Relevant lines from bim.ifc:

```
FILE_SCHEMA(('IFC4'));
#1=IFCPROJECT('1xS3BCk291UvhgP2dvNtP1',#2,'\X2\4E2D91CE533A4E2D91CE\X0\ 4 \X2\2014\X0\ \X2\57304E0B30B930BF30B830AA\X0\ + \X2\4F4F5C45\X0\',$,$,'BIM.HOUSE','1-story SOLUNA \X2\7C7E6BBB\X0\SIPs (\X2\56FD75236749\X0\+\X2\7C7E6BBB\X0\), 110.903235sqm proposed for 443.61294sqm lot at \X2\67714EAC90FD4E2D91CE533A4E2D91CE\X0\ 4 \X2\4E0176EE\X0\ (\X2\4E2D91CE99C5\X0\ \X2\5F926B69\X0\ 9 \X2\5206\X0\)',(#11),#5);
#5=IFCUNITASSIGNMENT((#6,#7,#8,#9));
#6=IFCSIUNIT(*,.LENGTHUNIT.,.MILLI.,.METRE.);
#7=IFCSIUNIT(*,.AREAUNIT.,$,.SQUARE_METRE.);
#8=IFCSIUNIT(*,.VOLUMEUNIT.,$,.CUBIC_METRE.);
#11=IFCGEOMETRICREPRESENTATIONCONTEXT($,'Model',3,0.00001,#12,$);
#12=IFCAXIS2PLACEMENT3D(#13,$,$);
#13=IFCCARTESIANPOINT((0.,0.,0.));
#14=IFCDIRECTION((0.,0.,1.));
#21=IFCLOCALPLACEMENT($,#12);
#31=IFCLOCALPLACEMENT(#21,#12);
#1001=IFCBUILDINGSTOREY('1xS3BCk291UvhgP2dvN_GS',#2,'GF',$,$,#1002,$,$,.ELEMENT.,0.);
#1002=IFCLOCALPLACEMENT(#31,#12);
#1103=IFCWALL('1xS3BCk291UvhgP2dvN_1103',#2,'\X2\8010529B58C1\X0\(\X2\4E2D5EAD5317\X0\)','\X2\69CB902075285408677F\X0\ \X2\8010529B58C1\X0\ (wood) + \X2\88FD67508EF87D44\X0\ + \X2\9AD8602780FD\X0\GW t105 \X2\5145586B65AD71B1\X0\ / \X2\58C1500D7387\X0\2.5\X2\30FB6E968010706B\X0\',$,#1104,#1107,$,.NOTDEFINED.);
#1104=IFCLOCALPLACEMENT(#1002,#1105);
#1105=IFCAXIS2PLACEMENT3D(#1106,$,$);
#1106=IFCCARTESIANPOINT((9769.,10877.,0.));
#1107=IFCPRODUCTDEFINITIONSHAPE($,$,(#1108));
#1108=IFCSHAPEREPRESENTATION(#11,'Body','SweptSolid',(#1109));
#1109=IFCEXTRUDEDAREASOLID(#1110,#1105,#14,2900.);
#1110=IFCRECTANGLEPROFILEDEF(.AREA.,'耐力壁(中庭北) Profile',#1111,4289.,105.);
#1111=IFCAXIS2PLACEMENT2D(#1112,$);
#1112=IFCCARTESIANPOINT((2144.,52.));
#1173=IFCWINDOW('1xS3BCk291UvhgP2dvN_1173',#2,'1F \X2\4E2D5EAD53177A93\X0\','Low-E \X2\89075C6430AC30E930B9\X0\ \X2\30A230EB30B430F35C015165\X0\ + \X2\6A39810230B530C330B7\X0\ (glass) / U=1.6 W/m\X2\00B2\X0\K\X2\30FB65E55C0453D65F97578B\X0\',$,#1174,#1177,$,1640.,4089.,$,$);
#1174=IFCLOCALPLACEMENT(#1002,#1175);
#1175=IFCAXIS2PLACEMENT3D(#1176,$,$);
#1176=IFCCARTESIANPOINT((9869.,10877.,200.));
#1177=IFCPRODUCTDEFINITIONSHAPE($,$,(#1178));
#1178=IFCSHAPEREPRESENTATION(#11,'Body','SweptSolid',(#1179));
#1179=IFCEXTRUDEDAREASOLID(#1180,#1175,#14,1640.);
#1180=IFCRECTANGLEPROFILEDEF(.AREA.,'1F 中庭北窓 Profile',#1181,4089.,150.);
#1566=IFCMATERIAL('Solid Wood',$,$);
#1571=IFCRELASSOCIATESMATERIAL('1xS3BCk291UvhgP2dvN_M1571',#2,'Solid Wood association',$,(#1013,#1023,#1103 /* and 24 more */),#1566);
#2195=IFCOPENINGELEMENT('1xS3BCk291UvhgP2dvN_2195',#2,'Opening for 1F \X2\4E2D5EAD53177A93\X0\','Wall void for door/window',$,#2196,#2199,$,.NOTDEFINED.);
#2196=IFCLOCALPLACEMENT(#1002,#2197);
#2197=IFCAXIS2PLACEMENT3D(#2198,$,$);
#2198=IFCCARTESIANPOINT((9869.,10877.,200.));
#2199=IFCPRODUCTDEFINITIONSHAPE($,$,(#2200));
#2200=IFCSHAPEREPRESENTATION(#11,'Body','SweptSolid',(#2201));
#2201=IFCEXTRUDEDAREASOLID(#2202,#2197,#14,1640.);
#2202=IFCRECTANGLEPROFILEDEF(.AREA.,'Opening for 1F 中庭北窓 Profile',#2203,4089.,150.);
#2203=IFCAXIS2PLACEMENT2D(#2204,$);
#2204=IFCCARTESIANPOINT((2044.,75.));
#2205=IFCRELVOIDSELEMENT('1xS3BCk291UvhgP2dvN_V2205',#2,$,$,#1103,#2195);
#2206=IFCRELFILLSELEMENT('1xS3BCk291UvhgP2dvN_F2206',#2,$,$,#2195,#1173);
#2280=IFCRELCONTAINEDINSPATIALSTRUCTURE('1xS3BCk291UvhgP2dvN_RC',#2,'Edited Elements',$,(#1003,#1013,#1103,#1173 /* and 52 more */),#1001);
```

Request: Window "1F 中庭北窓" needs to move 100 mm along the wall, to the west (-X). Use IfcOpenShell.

```python
import ifcopenshell
import ifcopenshell.api.geometry
import ifcopenshell.util.placement

model = ifcopenshell.open("bim.ifc")

window = model.by_guid("1xS3BCk291UvhgP2dvN_1173")
opening = window.FillsVoids[0].RelatingOpeningElement
wall = opening.VoidsElements[0].RelatingBuildingElement

wall_matrix = ifcopenshell.util.placement.get_local_placement(wall.ObjectPlacement)
shift = wall_matrix[:3, 0] * -100.0
before = ifcopenshell.util.placement.get_local_placement(window.ObjectPlacement)[:3, 3].copy()

# The window is not placed relative to its opening, so move both.
for product in (opening, window):
    matrix = ifcopenshell.util.placement.get_local_placement(product.ObjectPlacement)
    matrix[:3, 3] += shift
    ifcopenshell.api.geometry.edit_object_placement(model, product=product, matrix=matrix, is_si=False)

after = ifcopenshell.util.placement.get_local_placement(window.ObjectPlacement)[:3, 3]
print("window moved by", (after - before).round(3) + 0.0)

model.write("bim-out.ifc")
```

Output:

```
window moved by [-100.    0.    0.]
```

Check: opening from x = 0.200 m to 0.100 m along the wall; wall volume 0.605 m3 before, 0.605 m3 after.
